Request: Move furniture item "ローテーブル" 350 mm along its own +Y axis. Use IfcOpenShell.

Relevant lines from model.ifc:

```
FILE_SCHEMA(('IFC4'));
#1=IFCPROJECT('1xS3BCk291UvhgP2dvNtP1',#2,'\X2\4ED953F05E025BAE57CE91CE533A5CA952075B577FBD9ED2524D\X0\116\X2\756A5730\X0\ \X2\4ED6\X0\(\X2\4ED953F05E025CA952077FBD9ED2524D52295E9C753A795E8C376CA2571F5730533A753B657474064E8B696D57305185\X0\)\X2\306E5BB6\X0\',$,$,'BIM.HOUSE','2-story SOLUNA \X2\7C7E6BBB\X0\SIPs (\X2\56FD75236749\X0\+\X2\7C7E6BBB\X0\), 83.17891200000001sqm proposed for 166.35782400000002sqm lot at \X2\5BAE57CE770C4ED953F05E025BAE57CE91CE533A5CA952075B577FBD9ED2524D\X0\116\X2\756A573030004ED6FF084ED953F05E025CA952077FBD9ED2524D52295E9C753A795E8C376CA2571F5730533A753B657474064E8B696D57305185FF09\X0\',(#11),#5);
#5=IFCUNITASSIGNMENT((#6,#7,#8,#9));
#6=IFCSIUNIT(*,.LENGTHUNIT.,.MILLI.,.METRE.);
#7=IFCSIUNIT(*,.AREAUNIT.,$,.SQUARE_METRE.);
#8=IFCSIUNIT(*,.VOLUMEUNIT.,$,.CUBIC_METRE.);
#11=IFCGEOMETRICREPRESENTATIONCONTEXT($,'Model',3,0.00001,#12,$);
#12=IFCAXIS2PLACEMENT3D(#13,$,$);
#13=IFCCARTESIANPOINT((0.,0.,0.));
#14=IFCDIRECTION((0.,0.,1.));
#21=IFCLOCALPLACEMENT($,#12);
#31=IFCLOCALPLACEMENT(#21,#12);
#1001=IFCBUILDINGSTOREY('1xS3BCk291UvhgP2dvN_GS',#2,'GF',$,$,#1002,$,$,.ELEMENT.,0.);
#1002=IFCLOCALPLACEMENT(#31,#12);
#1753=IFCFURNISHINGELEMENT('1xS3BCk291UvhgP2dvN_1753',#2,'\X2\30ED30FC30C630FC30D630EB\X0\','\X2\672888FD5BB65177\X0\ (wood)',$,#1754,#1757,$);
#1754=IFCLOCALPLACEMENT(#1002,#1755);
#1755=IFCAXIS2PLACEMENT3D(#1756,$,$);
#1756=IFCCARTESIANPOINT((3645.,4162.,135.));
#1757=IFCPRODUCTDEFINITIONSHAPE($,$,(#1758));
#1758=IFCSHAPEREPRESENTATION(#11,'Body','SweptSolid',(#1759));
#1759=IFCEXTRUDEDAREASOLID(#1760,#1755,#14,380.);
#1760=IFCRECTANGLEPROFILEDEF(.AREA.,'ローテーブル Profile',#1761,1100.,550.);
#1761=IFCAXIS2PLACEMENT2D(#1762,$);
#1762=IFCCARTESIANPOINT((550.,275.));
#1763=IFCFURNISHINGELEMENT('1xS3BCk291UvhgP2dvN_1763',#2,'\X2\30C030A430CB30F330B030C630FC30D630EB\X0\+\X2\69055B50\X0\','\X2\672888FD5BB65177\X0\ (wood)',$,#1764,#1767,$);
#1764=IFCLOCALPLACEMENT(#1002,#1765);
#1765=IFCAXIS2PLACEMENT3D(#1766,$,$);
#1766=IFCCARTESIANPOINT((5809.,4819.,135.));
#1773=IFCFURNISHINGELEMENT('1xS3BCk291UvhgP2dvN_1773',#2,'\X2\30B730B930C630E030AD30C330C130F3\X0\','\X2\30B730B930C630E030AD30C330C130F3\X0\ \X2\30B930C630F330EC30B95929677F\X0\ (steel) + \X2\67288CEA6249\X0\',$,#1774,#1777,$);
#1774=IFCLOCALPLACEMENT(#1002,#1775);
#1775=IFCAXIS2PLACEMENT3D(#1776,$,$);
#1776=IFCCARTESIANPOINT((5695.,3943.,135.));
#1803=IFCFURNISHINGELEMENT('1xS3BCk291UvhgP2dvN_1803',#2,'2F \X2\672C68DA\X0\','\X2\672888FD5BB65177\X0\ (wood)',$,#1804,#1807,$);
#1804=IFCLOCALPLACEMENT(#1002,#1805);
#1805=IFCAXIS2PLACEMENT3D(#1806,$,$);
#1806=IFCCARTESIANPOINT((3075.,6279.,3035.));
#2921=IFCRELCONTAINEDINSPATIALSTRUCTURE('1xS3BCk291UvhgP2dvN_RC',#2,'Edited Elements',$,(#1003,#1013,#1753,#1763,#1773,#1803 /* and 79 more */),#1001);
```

```python
import ifcopenshell
import ifcopenshell.api.geometry
import ifcopenshell.util.placement
import ifcopenshell.util.unit

model = ifcopenshell.open("model.ifc")
unit_scale = ifcopenshell.util.unit.calculate_unit_scale(model)

item = model.by_id(1753)
matrix = ifcopenshell.util.placement.get_local_placement(item.ObjectPlacement)
matrix[:3, 3] += matrix[:3, 1] * 0.35 / unit_scale
ifcopenshell.api.geometry.edit_object_placement(model, product=item, matrix=matrix, is_si=False)

print(ifcopenshell.util.placement.get_local_placement(item.ObjectPlacement).round(3) + 0.0)

model.write("model_updated.ifc")
```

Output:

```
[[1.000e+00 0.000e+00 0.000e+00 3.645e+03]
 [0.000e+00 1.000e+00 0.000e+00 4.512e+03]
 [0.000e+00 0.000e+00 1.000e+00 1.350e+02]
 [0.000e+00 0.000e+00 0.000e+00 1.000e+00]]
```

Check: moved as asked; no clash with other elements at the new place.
